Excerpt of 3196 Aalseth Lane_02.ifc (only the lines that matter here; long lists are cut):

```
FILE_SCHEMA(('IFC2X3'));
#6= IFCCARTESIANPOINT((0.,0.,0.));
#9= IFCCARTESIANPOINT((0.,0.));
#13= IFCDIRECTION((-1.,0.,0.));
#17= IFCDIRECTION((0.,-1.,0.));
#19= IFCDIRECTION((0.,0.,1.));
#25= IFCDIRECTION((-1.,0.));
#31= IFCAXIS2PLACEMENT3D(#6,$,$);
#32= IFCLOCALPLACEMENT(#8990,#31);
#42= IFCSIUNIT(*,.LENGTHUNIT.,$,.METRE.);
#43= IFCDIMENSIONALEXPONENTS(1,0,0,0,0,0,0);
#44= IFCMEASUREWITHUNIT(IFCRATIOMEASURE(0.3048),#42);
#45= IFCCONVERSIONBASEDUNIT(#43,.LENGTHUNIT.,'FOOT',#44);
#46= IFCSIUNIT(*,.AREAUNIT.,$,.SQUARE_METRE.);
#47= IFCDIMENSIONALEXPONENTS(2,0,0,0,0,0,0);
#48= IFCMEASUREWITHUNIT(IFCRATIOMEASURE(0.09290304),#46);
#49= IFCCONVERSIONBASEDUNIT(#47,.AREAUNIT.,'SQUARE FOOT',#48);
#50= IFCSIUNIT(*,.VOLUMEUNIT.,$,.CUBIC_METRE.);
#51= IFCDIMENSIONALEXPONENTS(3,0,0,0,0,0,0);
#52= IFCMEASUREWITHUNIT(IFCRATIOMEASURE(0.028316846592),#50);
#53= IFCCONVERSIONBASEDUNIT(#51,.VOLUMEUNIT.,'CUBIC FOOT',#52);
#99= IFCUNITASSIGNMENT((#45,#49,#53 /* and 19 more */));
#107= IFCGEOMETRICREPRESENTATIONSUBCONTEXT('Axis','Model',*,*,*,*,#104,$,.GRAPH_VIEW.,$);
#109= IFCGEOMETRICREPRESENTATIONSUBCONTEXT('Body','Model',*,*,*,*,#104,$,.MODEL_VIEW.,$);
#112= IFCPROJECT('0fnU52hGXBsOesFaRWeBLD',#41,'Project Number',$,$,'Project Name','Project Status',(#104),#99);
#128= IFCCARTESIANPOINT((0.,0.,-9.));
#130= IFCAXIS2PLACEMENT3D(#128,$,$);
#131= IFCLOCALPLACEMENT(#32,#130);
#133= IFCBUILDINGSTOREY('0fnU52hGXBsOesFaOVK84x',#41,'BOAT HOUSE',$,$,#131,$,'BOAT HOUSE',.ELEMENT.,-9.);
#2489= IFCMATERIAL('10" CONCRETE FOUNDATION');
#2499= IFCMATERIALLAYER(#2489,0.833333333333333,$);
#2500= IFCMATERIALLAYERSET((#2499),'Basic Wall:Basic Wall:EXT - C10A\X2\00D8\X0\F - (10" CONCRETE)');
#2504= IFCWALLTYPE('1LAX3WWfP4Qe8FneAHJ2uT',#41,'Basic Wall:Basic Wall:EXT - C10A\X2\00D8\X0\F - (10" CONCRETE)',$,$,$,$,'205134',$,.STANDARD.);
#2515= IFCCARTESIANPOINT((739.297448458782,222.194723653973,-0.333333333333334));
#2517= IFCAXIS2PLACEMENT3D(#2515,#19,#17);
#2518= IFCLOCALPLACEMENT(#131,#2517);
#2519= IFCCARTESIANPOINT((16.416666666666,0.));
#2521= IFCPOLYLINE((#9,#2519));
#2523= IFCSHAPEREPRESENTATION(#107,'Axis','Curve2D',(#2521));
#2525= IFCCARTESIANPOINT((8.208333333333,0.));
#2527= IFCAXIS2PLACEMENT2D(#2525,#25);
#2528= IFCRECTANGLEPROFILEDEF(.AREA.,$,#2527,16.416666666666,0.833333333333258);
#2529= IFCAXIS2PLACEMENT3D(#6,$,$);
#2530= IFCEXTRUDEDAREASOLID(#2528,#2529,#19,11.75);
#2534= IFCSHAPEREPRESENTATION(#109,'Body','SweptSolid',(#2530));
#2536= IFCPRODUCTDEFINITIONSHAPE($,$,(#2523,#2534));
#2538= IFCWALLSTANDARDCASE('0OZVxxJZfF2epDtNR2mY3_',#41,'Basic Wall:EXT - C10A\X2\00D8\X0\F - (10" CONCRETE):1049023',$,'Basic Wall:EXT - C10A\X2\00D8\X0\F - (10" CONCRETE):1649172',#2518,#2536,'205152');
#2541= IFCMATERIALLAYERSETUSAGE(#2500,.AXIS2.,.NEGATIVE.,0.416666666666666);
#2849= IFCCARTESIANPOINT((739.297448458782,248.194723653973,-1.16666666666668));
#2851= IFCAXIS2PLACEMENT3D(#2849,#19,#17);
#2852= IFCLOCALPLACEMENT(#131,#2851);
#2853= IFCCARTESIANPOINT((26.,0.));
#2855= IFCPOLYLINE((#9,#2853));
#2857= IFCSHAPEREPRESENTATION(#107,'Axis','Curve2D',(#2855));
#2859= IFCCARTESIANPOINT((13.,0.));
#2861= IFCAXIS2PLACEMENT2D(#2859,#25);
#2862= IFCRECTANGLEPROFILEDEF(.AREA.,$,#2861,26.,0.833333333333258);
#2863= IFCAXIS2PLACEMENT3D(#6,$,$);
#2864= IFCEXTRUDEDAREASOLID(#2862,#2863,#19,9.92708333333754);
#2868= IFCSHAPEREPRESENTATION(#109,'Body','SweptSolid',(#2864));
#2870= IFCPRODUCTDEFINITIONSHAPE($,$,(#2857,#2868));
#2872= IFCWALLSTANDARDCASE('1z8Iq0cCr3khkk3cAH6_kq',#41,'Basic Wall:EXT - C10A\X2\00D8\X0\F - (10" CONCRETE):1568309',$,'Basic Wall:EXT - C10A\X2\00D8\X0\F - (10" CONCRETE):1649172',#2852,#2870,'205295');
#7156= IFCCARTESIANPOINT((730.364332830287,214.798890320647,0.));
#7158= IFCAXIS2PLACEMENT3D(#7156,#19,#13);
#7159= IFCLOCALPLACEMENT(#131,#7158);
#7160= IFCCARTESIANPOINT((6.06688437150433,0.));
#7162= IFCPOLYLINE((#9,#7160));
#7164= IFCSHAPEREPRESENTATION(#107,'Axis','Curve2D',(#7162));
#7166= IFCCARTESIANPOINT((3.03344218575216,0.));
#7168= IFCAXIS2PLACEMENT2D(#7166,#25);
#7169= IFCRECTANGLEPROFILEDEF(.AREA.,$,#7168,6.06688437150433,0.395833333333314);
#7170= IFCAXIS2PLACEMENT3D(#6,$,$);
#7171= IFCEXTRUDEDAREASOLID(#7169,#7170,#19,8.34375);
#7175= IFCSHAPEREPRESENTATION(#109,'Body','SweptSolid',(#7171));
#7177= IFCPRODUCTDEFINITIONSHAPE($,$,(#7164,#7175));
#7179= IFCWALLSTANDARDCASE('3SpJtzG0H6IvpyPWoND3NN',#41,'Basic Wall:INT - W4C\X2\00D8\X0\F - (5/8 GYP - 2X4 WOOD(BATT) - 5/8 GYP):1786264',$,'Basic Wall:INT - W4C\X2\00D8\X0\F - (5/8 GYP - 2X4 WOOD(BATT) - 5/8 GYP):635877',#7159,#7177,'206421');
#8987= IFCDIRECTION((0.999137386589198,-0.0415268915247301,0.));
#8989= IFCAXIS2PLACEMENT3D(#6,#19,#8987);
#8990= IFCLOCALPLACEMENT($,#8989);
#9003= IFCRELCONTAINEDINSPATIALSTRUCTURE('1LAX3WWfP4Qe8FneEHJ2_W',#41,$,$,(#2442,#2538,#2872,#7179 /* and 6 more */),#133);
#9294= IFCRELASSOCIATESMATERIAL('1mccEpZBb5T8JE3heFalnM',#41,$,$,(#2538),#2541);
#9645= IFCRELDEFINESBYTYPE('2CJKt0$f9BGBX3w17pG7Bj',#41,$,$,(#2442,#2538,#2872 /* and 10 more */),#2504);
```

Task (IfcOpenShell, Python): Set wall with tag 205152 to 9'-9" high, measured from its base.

```python
import ifcopenshell
import ifcopenshell.geom
import ifcopenshell.util.representation
import ifcopenshell.util.shape
import ifcopenshell.util.unit

model = ifcopenshell.open("3196 Aalseth Lane_02.ifc")
unit_scale = ifcopenshell.util.unit.calculate_unit_scale(model)
settings = ifcopenshell.geom.settings()


def volume(element):
    """Net volume in cubic metres, openings subtracted."""
    shape = ifcopenshell.geom.create_shape(settings, element)
    return ifcopenshell.util.shape.get_volume(shape.geometry)


wall = model.by_guid("0OZVxxJZfF2epDtNR2mY3_")
before = volume(wall)

body = ifcopenshell.util.representation.get_representation(wall, "Model", "Body")
solid = body.Items[0]
old_height = solid.Depth
solid.Depth = 117 * 0.0254 / unit_scale
after = volume(wall)

print(f"height {old_height:g} -> {solid.Depth:g}, volume {before:.3f} -> {after:.3f} m3")

model.write("3196 Aalseth Lane_02_v2.ifc")
```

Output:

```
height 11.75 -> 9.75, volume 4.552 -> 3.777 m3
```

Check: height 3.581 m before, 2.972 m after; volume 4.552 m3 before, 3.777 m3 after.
